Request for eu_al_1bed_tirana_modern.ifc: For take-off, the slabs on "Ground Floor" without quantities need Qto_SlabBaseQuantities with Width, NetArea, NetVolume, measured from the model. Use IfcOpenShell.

First a look at what the model holds.

```python
import ifcopenshell
import ifcopenshell.util.element
import ifcopenshell.util.unit

model = ifcopenshell.open("eu_al_1bed_tirana_modern.ifc")
print(model.schema)
for unit_type in ("LENGTHUNIT", "AREAUNIT", "VOLUMEUNIT"):
    print(unit_type, ifcopenshell.util.unit.calculate_unit_scale(model, unit_type))
storey = next(s for s in model.by_type("IfcBuildingStorey") if s.Name == "Ground Floor")
slabs = [e for e in ifcopenshell.util.element.get_decomposition(storey) if e.is_a("IfcSlab")]
for e in sorted(slabs, key=lambda e: e.id()):
    print(e.id(), e.is_a(), e.Name, list(ifcopenshell.util.element.get_psets(e, qtos_only=True)), sep=" | ")
```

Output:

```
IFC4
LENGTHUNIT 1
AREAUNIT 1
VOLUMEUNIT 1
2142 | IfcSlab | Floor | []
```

```python
import ifcopenshell
import ifcopenshell.api.pset
import ifcopenshell.geom
import ifcopenshell.util.element
import ifcopenshell.util.shape
import ifcopenshell.util.unit

model = ifcopenshell.open("eu_al_1bed_tirana_modern.ifc")
unit_scale = ifcopenshell.util.unit.calculate_unit_scale(model)
area_scale = ifcopenshell.util.unit.calculate_unit_scale(model, "AREAUNIT")
volume_scale = ifcopenshell.util.unit.calculate_unit_scale(model, "VOLUMEUNIT")
settings = ifcopenshell.geom.settings()

storey = next(s for s in model.by_type("IfcBuildingStorey") if s.Name == "Ground Floor")
slabs = [e for e in ifcopenshell.util.element.get_decomposition(storey) if e.is_a("IfcSlab")]

for e in sorted(slabs, key=lambda e: e.id()):
    if ifcopenshell.util.element.get_psets(e, qtos_only=True, should_inherit=False):
        continue
    # Geometry comes back in metres, in the element's own axes.
    shape = ifcopenshell.geom.create_shape(settings, e)
    values = {
        "Width": ifcopenshell.util.shape.get_z(shape.geometry) / unit_scale,
        "NetArea": ifcopenshell.util.shape.get_footprint_area(shape.geometry) / area_scale,
        "NetVolume": ifcopenshell.util.shape.get_volume(shape.geometry) / volume_scale,
    }
    qto = ifcopenshell.api.pset.add_qto(model, product=e, name="Qto_SlabBaseQuantities")
    ifcopenshell.api.pset.edit_qto(model, qto=qto, properties=values)
    print(e.id(), {k: round(v, 3) for k, v in values.items()})

model.write("eu_al_1bed_tirana_modern_rev.ifc")
```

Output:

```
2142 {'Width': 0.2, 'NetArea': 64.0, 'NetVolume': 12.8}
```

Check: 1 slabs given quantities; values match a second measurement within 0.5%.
